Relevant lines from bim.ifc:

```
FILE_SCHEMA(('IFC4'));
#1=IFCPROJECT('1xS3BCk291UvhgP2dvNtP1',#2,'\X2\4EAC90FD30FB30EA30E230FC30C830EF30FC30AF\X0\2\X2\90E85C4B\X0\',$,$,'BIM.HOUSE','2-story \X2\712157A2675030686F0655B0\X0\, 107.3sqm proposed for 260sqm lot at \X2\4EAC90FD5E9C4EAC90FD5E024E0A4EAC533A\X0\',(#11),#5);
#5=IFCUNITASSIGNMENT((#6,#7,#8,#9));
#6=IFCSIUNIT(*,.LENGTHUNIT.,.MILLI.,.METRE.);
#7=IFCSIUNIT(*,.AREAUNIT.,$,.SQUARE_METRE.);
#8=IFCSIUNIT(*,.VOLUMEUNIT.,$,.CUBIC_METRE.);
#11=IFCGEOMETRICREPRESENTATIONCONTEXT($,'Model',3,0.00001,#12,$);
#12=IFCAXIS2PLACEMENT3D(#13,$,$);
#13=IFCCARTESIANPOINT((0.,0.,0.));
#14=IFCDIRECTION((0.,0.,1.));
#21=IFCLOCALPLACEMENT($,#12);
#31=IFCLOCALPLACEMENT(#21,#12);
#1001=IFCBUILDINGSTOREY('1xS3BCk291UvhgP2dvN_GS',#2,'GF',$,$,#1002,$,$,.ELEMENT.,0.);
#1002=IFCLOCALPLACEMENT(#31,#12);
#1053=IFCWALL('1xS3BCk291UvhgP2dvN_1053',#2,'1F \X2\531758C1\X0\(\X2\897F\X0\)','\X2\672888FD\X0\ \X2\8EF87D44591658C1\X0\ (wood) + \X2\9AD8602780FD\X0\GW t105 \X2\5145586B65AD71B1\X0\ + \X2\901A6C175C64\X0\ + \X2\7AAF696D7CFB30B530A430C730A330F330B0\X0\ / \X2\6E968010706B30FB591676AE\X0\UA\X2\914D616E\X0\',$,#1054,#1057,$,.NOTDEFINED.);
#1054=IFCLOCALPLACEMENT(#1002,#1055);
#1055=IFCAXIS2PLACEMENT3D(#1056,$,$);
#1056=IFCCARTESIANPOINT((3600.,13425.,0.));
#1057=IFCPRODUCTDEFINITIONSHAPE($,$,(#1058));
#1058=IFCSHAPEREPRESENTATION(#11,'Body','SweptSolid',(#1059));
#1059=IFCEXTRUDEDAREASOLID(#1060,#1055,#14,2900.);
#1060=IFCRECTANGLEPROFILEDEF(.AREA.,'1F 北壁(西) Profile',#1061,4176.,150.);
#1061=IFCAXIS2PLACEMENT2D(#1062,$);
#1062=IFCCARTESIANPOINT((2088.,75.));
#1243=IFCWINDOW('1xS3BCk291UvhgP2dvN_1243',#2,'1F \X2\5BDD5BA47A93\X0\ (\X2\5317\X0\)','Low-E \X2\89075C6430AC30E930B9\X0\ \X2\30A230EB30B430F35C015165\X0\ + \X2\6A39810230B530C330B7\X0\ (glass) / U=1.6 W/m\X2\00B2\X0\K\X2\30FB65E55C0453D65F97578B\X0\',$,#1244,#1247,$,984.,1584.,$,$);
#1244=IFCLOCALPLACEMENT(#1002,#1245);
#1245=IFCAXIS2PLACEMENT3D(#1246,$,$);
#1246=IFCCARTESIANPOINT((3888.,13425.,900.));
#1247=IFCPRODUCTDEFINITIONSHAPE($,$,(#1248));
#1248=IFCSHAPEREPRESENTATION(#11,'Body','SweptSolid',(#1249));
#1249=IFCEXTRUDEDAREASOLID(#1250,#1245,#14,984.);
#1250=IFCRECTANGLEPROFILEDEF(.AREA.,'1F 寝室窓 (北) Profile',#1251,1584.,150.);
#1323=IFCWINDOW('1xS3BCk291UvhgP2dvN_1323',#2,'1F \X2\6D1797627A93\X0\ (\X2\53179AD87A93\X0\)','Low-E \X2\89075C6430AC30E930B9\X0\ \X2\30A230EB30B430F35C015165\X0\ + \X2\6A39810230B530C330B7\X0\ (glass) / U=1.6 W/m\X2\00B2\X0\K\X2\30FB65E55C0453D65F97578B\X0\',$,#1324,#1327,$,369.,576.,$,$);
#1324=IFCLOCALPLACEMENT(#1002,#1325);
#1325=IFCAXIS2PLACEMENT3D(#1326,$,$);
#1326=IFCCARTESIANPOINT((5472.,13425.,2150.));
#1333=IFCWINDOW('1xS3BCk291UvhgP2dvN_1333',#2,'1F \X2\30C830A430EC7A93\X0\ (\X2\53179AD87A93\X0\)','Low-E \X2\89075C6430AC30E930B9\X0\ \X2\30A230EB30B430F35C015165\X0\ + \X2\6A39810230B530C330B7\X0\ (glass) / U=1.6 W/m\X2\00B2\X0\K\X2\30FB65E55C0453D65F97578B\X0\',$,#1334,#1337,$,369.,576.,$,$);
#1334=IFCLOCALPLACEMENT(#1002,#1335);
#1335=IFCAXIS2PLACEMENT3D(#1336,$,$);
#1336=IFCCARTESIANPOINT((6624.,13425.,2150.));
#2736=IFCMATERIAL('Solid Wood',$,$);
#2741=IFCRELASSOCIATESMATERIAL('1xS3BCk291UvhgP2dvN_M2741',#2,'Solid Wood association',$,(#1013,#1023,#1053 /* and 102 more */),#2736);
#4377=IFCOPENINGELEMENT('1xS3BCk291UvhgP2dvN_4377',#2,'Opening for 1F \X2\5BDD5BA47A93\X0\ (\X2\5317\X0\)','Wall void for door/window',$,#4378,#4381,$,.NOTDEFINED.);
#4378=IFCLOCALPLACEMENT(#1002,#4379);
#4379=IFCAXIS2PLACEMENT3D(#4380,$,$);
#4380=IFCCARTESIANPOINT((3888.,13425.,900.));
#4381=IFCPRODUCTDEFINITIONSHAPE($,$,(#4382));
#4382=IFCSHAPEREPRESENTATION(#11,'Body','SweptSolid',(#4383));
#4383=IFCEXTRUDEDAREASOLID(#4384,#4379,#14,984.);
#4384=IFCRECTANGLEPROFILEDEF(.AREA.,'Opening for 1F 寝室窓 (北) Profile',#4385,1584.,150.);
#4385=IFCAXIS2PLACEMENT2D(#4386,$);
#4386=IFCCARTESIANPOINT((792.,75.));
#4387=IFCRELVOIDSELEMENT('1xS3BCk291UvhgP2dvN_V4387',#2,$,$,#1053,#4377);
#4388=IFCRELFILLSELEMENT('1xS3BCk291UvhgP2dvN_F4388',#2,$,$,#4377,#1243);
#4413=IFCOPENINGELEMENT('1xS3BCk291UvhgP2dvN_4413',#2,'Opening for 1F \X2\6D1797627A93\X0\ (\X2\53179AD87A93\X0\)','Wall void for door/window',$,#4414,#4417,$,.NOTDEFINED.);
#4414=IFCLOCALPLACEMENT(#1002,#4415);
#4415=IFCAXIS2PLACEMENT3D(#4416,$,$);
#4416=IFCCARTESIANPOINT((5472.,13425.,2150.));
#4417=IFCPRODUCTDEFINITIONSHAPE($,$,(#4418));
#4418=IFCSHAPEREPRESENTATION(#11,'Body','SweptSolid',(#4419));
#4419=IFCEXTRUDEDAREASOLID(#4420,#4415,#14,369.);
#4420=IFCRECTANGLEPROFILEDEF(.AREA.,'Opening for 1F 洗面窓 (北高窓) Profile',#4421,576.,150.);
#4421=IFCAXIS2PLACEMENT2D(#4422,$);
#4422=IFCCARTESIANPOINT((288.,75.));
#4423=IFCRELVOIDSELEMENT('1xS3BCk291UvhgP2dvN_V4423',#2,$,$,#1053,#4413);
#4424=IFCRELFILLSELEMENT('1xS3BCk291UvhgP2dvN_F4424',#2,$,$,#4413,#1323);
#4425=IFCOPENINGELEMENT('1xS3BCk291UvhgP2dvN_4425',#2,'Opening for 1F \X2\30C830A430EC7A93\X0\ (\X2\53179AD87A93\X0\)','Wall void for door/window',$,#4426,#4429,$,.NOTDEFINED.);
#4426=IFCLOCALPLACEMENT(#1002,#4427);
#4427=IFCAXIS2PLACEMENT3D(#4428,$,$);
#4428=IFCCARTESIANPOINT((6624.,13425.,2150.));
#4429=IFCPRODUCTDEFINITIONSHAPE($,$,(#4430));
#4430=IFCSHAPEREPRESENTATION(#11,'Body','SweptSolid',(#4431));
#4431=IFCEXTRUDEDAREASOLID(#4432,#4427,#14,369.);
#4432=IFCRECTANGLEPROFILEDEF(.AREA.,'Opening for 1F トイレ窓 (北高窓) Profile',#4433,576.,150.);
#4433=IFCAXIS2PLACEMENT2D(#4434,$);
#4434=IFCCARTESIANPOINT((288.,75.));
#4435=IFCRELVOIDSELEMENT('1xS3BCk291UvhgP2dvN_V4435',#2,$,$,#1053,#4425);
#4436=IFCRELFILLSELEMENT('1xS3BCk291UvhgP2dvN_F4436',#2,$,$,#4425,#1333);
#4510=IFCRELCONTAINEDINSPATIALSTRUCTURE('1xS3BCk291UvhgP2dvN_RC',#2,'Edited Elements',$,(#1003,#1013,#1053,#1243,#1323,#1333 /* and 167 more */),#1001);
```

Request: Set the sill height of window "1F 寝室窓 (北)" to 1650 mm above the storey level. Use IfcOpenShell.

```python
import numpy as np
import ifcopenshell
import ifcopenshell.api.geometry
import ifcopenshell.geom
import ifcopenshell.util.element
import ifcopenshell.util.placement
import ifcopenshell.util.shape
import ifcopenshell.util.unit

model = ifcopenshell.open("bim.ifc")
unit_scale = ifcopenshell.util.unit.calculate_unit_scale(model)

window = model.by_guid("1xS3BCk291UvhgP2dvN_1243")
opening = window.FillsVoids[0].RelatingOpeningElement
storey = ifcopenshell.util.element.get_container(window, ifc_class="IfcBuildingStorey")
level = ifcopenshell.util.placement.get_local_placement(storey.ObjectPlacement)[2, 3]

# The opening's origin need not be at the sill, so measure its lowest point.
shape = ifcopenshell.geom.create_shape(ifcopenshell.geom.settings(), opening)
bottom = ifcopenshell.util.shape.get_shape_bottom_elevation(shape, shape.geometry) / unit_scale
dz = level + 1650.0 - bottom

shift = np.array([0.0, 0.0, dz])
# The window is not placed relative to its opening, so move both.
for product in (opening, window):
    matrix = ifcopenshell.util.placement.get_local_placement(product.ObjectPlacement)
    matrix[:3, 3] += shift
    ifcopenshell.api.geometry.edit_object_placement(model, product=product, matrix=matrix, is_si=False)

print(f"moved by {dz * unit_scale:+.3f} m")

model.write("bim_updated.ifc")
```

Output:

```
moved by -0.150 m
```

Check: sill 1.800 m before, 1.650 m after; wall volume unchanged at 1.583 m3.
